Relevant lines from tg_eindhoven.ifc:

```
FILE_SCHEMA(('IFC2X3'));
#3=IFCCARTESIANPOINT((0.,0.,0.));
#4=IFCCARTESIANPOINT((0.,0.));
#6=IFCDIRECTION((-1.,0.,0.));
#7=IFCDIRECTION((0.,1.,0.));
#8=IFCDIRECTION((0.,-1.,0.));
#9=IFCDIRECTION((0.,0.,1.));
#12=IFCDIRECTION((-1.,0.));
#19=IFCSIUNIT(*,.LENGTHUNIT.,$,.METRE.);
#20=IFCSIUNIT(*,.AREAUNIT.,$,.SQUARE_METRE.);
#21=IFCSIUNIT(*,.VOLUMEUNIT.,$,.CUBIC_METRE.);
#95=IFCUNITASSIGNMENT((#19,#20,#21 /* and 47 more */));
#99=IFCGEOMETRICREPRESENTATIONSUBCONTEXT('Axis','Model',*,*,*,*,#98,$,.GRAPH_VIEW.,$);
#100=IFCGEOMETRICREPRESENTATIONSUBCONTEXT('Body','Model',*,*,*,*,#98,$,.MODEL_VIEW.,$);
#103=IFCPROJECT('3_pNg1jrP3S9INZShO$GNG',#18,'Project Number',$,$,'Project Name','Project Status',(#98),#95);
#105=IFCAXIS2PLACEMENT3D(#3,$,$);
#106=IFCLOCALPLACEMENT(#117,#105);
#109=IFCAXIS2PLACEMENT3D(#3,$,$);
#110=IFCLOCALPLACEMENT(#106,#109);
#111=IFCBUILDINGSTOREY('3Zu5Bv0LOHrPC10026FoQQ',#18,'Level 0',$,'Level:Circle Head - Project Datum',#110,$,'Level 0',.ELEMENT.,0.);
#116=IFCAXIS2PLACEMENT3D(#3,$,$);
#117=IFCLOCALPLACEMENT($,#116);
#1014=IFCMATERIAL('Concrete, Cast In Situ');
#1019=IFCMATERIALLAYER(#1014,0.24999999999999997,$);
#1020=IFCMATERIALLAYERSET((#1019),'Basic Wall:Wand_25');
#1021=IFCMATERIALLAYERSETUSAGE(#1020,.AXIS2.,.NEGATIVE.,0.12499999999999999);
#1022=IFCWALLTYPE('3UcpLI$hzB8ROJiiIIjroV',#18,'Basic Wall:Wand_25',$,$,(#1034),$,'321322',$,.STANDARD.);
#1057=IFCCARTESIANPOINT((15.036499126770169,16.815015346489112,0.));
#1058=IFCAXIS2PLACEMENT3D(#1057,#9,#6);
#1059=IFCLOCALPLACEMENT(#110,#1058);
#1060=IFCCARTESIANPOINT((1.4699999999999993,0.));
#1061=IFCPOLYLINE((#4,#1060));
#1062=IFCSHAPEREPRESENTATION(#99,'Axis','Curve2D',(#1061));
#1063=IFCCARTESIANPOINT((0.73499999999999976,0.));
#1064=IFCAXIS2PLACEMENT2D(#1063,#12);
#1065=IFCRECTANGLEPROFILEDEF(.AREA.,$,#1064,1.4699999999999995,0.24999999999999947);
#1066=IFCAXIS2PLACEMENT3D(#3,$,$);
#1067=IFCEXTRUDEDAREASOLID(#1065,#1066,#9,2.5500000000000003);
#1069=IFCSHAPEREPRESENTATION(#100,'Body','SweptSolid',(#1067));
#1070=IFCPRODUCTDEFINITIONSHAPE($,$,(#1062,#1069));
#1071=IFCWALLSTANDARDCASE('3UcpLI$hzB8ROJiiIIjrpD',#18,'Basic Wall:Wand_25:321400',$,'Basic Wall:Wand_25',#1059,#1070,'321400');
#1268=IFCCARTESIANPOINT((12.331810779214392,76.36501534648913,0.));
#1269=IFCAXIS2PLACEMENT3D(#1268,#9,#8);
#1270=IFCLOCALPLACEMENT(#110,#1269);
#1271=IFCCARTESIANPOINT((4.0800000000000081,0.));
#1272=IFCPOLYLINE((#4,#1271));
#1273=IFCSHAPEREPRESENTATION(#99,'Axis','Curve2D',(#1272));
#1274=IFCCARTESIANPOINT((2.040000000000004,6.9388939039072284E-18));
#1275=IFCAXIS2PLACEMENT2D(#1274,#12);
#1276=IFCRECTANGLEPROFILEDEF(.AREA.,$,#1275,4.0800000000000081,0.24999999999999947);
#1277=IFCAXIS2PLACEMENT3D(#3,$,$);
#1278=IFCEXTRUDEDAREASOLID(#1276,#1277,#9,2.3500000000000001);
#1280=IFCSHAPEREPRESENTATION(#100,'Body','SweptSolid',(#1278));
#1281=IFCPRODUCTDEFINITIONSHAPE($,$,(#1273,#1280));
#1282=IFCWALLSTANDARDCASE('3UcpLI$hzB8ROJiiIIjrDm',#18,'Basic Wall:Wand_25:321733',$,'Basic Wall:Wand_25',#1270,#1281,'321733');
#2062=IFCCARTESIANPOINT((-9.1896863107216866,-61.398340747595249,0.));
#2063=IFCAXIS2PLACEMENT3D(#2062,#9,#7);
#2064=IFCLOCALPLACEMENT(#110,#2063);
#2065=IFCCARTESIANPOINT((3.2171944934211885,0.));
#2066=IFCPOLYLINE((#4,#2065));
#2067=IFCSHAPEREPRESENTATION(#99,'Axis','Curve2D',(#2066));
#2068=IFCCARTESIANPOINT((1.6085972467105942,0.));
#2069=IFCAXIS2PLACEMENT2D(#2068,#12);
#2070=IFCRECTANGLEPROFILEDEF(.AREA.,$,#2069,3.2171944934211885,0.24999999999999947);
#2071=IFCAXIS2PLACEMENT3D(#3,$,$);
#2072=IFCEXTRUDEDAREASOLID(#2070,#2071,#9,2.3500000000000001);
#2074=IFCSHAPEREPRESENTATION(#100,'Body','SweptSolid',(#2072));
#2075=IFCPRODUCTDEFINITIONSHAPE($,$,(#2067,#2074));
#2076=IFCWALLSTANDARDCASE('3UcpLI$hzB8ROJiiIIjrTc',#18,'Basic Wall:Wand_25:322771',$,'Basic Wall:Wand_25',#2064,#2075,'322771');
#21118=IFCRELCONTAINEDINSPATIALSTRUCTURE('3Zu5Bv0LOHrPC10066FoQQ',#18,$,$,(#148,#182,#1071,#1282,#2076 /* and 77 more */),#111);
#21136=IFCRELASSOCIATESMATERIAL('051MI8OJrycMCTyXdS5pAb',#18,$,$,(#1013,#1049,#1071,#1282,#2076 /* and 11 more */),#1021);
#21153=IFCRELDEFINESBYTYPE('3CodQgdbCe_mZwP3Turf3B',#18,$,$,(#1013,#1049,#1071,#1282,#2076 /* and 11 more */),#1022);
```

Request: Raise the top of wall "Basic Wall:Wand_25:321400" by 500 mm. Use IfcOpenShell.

```python
import ifcopenshell
import ifcopenshell.geom
import ifcopenshell.util.representation
import ifcopenshell.util.shape

model = ifcopenshell.open("tg_eindhoven.ifc")
settings = ifcopenshell.geom.settings()


def volume(element):
    """Net volume in cubic metres, openings subtracted."""
    shape = ifcopenshell.geom.create_shape(settings, element)
    return ifcopenshell.util.shape.get_volume(shape.geometry)


wall = model.by_guid("3UcpLI$hzB8ROJiiIIjrpD")
before = volume(wall)

body = ifcopenshell.util.representation.get_representation(wall, "Model", "Body")
solid = body.Items[0]
old_height = solid.Depth
solid.Depth += 0.5
after = volume(wall)

print(f"height {old_height:g} -> {solid.Depth:g}, volume {before:.3f} -> {after:.3f} m3")

model.write("tg_eindhoven_v2.ifc")
```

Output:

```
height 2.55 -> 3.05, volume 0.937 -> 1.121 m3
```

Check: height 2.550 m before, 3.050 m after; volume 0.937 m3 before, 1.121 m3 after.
